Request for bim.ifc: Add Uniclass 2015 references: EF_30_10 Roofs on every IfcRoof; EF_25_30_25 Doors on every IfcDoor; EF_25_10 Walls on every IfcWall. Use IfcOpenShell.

First a look at what the model holds.

```python
import ifcopenshell

model = ifcopenshell.open("bim.ifc")
print(model.schema)
print("classifications:", [c.Name for c in model.by_type("IfcClassification")])
for ifc_class in ("IfcDoor", "IfcRoof", "IfcStair", "IfcWall", "IfcWindow"):
    print(ifc_class, len(model.by_type(ifc_class)))
```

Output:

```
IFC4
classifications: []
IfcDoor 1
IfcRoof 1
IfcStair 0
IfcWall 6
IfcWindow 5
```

```python
import ifcopenshell
import ifcopenshell.api.classification

model = ifcopenshell.open("bim.ifc")

system = ifcopenshell.api.classification.add_classification(model, classification="Uniclass 2015")

codes = {
    "IfcRoof": ("EF_30_10", "Roofs"),
    "IfcDoor": ("EF_25_30_25", "Doors"),
    "IfcWall": ("EF_25_10", "Walls"),
}
for ifc_class, (code, name) in codes.items():
    products = model.by_type(ifc_class)
    ifcopenshell.api.classification.add_reference(
        model, products=products, classification=system, identification=code, name=name
    )
    print(code, len(products))

model.write("bim_v2.ifc")
```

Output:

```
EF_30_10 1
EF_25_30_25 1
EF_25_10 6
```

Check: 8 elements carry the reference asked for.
